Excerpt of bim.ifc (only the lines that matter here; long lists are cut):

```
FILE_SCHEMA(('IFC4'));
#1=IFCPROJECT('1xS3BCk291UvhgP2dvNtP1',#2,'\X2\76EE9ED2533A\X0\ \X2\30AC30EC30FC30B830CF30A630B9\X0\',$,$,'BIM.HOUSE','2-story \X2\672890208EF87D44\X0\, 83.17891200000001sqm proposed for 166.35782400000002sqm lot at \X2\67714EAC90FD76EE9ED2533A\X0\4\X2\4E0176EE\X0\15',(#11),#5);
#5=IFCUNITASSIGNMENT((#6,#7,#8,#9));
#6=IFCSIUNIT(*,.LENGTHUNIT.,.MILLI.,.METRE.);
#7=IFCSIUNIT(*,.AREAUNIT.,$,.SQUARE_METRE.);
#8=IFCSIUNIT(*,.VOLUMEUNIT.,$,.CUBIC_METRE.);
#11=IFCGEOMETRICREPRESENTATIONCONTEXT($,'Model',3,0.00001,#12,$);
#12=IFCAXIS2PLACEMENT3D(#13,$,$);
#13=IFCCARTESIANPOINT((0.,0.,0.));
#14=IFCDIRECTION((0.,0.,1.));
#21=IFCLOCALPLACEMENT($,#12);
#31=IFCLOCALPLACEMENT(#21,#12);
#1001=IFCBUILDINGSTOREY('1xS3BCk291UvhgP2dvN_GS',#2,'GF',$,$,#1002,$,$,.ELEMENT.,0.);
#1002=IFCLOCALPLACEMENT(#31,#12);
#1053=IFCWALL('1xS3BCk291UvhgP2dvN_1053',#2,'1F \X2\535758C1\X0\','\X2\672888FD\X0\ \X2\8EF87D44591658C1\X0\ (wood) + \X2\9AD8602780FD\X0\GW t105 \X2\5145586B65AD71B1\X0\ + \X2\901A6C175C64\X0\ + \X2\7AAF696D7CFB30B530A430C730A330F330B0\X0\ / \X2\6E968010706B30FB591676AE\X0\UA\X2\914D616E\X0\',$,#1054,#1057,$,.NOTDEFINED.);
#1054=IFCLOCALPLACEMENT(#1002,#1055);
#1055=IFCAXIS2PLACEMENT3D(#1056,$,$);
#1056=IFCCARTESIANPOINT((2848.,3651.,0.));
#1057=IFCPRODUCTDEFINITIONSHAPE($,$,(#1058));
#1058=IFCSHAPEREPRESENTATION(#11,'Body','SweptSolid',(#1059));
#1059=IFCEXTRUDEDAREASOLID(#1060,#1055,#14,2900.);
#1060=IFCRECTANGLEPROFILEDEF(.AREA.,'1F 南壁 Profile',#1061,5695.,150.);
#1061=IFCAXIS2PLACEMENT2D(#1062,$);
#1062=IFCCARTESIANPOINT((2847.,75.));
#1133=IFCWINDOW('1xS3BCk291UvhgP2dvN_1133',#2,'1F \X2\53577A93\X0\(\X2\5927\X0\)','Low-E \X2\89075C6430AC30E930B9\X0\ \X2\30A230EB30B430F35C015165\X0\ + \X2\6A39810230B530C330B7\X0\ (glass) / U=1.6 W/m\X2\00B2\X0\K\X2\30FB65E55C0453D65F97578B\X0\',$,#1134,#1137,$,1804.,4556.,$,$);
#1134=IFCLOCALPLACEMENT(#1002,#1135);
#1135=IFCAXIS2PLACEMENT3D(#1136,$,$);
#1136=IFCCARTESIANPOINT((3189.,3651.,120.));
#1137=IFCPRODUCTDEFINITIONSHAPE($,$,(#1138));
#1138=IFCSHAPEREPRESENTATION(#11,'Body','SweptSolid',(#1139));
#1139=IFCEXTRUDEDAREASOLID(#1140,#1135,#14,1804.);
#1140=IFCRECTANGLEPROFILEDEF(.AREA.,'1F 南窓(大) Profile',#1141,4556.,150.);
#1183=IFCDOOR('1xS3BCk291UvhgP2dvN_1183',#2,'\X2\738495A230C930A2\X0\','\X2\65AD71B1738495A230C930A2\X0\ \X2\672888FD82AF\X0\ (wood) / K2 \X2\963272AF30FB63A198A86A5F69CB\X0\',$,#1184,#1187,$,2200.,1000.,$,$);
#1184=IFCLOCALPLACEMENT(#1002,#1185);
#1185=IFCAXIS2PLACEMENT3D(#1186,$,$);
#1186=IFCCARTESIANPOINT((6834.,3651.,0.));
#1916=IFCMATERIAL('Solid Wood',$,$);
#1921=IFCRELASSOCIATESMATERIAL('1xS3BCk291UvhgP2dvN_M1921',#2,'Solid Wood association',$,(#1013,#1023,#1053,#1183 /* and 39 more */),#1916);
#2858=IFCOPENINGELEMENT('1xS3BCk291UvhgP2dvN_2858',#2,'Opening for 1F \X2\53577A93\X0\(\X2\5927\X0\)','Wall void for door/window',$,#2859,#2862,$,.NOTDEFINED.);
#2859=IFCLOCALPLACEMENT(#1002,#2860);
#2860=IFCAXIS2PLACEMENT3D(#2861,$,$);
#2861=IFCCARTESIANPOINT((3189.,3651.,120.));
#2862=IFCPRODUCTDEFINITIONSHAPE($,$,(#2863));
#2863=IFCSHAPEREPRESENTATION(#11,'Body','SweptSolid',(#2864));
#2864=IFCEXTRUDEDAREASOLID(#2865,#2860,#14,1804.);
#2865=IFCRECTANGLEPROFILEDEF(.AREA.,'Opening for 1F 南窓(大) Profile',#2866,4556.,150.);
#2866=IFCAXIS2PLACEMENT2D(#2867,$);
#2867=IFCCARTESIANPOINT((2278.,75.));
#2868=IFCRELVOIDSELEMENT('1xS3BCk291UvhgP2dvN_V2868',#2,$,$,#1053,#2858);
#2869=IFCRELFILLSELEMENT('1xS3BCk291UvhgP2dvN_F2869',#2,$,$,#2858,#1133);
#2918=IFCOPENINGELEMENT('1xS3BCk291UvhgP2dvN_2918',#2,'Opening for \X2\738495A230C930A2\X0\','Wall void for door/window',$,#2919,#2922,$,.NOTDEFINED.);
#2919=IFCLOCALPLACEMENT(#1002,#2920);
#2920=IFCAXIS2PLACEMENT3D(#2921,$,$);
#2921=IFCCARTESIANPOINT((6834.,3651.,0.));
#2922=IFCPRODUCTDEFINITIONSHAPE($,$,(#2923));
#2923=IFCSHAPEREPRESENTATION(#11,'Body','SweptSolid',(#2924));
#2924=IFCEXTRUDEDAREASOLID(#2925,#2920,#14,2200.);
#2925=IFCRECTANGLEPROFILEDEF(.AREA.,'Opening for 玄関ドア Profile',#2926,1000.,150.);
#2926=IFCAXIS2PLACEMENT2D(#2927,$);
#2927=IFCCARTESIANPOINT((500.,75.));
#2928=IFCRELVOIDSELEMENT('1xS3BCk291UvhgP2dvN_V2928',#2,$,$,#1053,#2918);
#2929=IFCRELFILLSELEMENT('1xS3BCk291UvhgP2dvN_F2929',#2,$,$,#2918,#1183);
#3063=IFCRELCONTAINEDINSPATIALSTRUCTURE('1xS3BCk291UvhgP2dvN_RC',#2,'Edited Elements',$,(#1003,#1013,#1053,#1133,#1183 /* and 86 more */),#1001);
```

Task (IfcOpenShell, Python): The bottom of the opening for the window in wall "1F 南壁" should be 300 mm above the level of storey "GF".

```python
import numpy as np
import ifcopenshell
import ifcopenshell.api.geometry
import ifcopenshell.geom
import ifcopenshell.util.element
import ifcopenshell.util.placement
import ifcopenshell.util.shape
import ifcopenshell.util.unit

model = ifcopenshell.open("bim.ifc")
unit_scale = ifcopenshell.util.unit.calculate_unit_scale(model)

window = model.by_guid("1xS3BCk291UvhgP2dvN_1133")
opening = window.FillsVoids[0].RelatingOpeningElement
storey = ifcopenshell.util.element.get_container(window, ifc_class="IfcBuildingStorey")
level = ifcopenshell.util.placement.get_local_placement(storey.ObjectPlacement)[2, 3]

# The opening's origin need not be at the sill, so measure its lowest point.
shape = ifcopenshell.geom.create_shape(ifcopenshell.geom.settings(), opening)
bottom = ifcopenshell.util.shape.get_shape_bottom_elevation(shape, shape.geometry) / unit_scale
dz = level + 300.0 - bottom

shift = np.array([0.0, 0.0, dz])
# The window is not placed relative to its opening, so move both.
for product in (opening, window):
    matrix = ifcopenshell.util.placement.get_local_placement(product.ObjectPlacement)
    matrix[:3, 3] += shift
    ifcopenshell.api.geometry.edit_object_placement(model, product=product, matrix=matrix, is_si=False)

print(f"moved by {dz * unit_scale:+.3f} m")

model.write("bim_rev.ifc")
```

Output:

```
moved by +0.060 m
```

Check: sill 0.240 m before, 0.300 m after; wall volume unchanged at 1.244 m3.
